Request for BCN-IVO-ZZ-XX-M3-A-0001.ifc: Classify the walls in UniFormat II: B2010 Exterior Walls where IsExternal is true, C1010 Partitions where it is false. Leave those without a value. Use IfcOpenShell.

First a look at what the model holds.

```python
import ifcopenshell
import ifcopenshell.util.element

model = ifcopenshell.open("BCN-IVO-ZZ-XX-M3-A-0001.ifc")
print(model.schema)
print("classifications:", [c.Name for c in model.by_type("IfcClassification")])
values = [ifcopenshell.util.element.get_pset(e, "Pset_WallCommon", "IsExternal") for e in model.by_type("IfcWall")]
for value in (True, False, None):
    print("IsExternal", value, values.count(value))
```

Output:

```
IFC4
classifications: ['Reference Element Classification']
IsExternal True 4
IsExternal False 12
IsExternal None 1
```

```python
import ifcopenshell
import ifcopenshell.api.classification
import ifcopenshell.util.element

model = ifcopenshell.open("BCN-IVO-ZZ-XX-M3-A-0001.ifc")

system = ifcopenshell.api.classification.add_classification(model, classification="UniFormat II")

walls = model.by_type("IfcWall")
external = {e: ifcopenshell.util.element.get_pset(e, "Pset_WallCommon", "IsExternal") for e in walls}
for flag, code, name in ((True, "B2010", "Exterior Walls"), (False, "C1010", "Partitions")):
    products = [e for e in walls if external[e] is flag]
    ifcopenshell.api.classification.add_reference(
        model, products=products, classification=system, identification=code, name=name
    )
    print(code, len(products))

model.write("BCN-IVO-ZZ-XX-M3-A-0001_updated.ifc")
```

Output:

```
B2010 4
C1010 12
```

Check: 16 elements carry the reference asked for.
